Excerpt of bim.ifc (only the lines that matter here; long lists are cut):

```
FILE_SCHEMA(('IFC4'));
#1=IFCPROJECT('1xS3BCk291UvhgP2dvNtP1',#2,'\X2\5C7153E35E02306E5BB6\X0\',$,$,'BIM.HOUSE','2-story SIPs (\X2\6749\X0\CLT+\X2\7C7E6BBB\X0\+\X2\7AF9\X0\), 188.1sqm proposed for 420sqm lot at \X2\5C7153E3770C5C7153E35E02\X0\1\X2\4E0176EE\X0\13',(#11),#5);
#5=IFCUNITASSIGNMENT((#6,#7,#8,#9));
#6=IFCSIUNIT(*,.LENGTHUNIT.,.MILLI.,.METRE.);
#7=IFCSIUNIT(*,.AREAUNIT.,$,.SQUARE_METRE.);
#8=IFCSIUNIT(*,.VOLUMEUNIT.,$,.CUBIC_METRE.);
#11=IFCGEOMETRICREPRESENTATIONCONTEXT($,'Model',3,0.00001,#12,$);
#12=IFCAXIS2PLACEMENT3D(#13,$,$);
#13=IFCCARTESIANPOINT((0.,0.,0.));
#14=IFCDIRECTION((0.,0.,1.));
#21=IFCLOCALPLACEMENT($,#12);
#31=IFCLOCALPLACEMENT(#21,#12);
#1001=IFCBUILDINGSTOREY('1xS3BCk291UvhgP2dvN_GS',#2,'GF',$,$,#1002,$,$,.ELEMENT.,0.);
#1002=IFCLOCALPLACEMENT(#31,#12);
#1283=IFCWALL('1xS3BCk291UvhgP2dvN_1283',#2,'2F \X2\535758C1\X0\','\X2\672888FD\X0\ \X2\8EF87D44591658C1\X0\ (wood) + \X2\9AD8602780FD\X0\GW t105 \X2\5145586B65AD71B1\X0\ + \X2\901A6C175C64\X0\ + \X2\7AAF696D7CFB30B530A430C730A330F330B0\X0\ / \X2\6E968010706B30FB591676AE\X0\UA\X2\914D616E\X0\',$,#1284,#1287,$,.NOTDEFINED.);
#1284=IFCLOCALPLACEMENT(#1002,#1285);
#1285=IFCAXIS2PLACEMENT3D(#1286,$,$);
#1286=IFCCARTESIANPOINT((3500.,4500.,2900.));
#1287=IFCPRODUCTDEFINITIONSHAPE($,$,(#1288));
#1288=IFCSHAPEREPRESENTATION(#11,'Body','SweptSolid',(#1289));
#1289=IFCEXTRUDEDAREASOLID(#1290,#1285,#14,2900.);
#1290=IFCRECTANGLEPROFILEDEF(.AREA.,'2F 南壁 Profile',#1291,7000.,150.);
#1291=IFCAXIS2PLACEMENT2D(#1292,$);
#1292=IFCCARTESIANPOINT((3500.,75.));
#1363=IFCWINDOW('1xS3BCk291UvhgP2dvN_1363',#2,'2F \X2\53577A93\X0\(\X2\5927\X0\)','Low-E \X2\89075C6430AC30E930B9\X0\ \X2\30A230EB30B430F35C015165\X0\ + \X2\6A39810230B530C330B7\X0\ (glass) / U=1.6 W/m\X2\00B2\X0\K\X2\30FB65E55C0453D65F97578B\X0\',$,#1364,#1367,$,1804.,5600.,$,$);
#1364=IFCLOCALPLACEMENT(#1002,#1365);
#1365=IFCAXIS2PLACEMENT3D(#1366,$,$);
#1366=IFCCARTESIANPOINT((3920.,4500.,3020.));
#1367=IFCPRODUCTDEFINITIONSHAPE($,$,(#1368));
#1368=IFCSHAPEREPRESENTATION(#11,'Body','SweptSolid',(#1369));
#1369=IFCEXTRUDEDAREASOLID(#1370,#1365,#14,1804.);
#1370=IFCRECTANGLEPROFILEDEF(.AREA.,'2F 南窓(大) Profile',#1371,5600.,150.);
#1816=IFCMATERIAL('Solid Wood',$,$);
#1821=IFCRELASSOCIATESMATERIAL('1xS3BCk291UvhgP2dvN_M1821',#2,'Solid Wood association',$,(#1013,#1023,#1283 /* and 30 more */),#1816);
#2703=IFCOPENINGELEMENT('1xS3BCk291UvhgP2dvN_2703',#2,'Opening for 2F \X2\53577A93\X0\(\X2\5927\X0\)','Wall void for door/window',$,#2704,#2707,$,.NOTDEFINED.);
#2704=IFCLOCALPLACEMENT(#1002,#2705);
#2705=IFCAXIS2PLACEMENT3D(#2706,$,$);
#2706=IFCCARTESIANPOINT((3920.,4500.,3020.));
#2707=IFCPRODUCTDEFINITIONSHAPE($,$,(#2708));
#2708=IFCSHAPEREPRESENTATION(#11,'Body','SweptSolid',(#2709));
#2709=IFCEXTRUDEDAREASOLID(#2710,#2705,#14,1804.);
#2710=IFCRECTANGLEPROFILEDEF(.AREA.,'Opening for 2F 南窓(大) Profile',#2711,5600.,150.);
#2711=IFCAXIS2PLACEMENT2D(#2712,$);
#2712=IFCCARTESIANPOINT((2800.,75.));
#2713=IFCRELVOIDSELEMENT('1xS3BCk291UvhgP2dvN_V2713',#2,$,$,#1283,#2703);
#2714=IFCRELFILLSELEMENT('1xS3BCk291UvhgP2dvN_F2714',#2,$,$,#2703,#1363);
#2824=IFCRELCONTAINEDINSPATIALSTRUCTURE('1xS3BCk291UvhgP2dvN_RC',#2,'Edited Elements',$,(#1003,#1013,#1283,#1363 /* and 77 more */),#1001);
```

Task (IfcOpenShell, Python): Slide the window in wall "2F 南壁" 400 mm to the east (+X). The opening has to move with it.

```python
import ifcopenshell
import ifcopenshell.api.geometry
import ifcopenshell.util.placement
import ifcopenshell.util.unit

model = ifcopenshell.open("bim.ifc")
unit_scale = ifcopenshell.util.unit.calculate_unit_scale(model)

window = model.by_id(1363)
opening = window.FillsVoids[0].RelatingOpeningElement
wall = opening.VoidsElements[0].RelatingBuildingElement

wall_matrix = ifcopenshell.util.placement.get_local_placement(wall.ObjectPlacement)
shift = wall_matrix[:3, 0] * 0.4 / unit_scale
before = ifcopenshell.util.placement.get_local_placement(window.ObjectPlacement)[:3, 3].copy()

# The window is not placed relative to its opening, so move both.
for product in (opening, window):
    matrix = ifcopenshell.util.placement.get_local_placement(product.ObjectPlacement)
    matrix[:3, 3] += shift
    ifcopenshell.api.geometry.edit_object_placement(model, product=product, matrix=matrix, is_si=False)

after = ifcopenshell.util.placement.get_local_placement(window.ObjectPlacement)[:3, 3]
print("window moved by", (after - before).round(3) + 0.0)

model.write("bim_rev.ifc")
```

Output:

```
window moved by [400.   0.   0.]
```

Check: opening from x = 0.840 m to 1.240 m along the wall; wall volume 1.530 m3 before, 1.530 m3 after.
